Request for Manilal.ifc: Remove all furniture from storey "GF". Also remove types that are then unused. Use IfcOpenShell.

First a look at what the model holds.

```python
import ifcopenshell
import ifcopenshell.util.element

model = ifcopenshell.open("Manilal.ifc")
print(model.schema)
storey = next(s for s in model.by_type("IfcBuildingStorey") if s.Name == "GF")
furniture = [e for e in ifcopenshell.util.element.get_decomposition(storey) if e.is_a("IfcFurnishingElement")]
seen = {}
for e in furniture:
    element_type = ifcopenshell.util.element.get_type(e)
    name = element_type.Name if element_type not in (None, e) else None
    seen[name] = seen.get(name, 0) + 1
for name, count in sorted(seen.items(), key=str):
    print(count, "x", name)
```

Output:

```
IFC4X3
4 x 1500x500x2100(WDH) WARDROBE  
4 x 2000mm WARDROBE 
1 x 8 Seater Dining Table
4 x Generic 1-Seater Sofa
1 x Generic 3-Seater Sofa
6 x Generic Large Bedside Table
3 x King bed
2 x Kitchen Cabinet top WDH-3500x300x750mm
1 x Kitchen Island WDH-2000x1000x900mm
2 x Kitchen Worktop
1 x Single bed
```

```python
import ifcopenshell
import ifcopenshell.api.root
import ifcopenshell.util.element

model = ifcopenshell.open("Manilal.ifc")

storey = next(s for s in model.by_type("IfcBuildingStorey") if s.Name == "GF")
furniture = [e for e in ifcopenshell.util.element.get_decomposition(storey) if e.is_a("IfcFurnishingElement")]
types = {ifcopenshell.util.element.get_type(e) for e in furniture} - {None, *furniture}

for e in furniture:
    ifcopenshell.api.root.remove_product(model, product=e)
print(len(furniture), "removed")

unused = [t for t in types if not ifcopenshell.util.element.get_types(t)]
for t in unused:
    ifcopenshell.api.root.remove_product(model, product=t)
print(len(unused), "unused types removed")

model.write("Manilal_edited.ifc")
```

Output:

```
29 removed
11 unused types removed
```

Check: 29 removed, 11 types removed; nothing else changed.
